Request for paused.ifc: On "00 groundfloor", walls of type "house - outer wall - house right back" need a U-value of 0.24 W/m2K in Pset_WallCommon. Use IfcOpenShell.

First a look at what the model holds.

```python
import ifcopenshell
import ifcopenshell.util.element

model = ifcopenshell.open("paused.ifc")
print(model.schema)
storey = next(s for s in model.by_type("IfcBuildingStorey") if s.Name == "00 groundfloor")
walls = [e for e in ifcopenshell.util.element.get_decomposition(storey) if e.is_a("IfcWall")]
seen = {}
for e in walls:
    element_type = ifcopenshell.util.element.get_type(e)
    key = (element_type.Name if element_type != e and element_type else None, ifcopenshell.util.element.get_pset(e, "Pset_WallCommon", "ThermalTransmittance"))
    seen[key] = seen.get(key, 0) + 1
for (name, value), count in sorted(seen.items(), key=str):
    print(count, "x", name, "|", value)
```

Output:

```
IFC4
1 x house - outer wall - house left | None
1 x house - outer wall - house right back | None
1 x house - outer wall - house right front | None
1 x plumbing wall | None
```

```python
import ifcopenshell
import ifcopenshell.api.pset
import ifcopenshell.util.element

model = ifcopenshell.open("paused.ifc")

storey = next(s for s in model.by_type("IfcBuildingStorey") if s.Name == "00 groundfloor")
walls = [e for e in ifcopenshell.util.element.get_decomposition(storey) if e.is_a("IfcWall")]

count = 0
for e in walls:
    element_type = ifcopenshell.util.element.get_type(e)
    if element_type in (None, e) or element_type.Name != "house - outer wall - house right back":
        continue
    # add_pset returns the element's existing set when there is one.
    pset = ifcopenshell.api.pset.add_pset(model, product=e, name="Pset_WallCommon")
    ifcopenshell.api.pset.edit_pset(model, pset=pset, properties={"ThermalTransmittance": 0.24})
    count += 1

print(count, "walls updated")

model.write("paused-out.ifc")
```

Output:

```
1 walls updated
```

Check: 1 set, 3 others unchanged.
